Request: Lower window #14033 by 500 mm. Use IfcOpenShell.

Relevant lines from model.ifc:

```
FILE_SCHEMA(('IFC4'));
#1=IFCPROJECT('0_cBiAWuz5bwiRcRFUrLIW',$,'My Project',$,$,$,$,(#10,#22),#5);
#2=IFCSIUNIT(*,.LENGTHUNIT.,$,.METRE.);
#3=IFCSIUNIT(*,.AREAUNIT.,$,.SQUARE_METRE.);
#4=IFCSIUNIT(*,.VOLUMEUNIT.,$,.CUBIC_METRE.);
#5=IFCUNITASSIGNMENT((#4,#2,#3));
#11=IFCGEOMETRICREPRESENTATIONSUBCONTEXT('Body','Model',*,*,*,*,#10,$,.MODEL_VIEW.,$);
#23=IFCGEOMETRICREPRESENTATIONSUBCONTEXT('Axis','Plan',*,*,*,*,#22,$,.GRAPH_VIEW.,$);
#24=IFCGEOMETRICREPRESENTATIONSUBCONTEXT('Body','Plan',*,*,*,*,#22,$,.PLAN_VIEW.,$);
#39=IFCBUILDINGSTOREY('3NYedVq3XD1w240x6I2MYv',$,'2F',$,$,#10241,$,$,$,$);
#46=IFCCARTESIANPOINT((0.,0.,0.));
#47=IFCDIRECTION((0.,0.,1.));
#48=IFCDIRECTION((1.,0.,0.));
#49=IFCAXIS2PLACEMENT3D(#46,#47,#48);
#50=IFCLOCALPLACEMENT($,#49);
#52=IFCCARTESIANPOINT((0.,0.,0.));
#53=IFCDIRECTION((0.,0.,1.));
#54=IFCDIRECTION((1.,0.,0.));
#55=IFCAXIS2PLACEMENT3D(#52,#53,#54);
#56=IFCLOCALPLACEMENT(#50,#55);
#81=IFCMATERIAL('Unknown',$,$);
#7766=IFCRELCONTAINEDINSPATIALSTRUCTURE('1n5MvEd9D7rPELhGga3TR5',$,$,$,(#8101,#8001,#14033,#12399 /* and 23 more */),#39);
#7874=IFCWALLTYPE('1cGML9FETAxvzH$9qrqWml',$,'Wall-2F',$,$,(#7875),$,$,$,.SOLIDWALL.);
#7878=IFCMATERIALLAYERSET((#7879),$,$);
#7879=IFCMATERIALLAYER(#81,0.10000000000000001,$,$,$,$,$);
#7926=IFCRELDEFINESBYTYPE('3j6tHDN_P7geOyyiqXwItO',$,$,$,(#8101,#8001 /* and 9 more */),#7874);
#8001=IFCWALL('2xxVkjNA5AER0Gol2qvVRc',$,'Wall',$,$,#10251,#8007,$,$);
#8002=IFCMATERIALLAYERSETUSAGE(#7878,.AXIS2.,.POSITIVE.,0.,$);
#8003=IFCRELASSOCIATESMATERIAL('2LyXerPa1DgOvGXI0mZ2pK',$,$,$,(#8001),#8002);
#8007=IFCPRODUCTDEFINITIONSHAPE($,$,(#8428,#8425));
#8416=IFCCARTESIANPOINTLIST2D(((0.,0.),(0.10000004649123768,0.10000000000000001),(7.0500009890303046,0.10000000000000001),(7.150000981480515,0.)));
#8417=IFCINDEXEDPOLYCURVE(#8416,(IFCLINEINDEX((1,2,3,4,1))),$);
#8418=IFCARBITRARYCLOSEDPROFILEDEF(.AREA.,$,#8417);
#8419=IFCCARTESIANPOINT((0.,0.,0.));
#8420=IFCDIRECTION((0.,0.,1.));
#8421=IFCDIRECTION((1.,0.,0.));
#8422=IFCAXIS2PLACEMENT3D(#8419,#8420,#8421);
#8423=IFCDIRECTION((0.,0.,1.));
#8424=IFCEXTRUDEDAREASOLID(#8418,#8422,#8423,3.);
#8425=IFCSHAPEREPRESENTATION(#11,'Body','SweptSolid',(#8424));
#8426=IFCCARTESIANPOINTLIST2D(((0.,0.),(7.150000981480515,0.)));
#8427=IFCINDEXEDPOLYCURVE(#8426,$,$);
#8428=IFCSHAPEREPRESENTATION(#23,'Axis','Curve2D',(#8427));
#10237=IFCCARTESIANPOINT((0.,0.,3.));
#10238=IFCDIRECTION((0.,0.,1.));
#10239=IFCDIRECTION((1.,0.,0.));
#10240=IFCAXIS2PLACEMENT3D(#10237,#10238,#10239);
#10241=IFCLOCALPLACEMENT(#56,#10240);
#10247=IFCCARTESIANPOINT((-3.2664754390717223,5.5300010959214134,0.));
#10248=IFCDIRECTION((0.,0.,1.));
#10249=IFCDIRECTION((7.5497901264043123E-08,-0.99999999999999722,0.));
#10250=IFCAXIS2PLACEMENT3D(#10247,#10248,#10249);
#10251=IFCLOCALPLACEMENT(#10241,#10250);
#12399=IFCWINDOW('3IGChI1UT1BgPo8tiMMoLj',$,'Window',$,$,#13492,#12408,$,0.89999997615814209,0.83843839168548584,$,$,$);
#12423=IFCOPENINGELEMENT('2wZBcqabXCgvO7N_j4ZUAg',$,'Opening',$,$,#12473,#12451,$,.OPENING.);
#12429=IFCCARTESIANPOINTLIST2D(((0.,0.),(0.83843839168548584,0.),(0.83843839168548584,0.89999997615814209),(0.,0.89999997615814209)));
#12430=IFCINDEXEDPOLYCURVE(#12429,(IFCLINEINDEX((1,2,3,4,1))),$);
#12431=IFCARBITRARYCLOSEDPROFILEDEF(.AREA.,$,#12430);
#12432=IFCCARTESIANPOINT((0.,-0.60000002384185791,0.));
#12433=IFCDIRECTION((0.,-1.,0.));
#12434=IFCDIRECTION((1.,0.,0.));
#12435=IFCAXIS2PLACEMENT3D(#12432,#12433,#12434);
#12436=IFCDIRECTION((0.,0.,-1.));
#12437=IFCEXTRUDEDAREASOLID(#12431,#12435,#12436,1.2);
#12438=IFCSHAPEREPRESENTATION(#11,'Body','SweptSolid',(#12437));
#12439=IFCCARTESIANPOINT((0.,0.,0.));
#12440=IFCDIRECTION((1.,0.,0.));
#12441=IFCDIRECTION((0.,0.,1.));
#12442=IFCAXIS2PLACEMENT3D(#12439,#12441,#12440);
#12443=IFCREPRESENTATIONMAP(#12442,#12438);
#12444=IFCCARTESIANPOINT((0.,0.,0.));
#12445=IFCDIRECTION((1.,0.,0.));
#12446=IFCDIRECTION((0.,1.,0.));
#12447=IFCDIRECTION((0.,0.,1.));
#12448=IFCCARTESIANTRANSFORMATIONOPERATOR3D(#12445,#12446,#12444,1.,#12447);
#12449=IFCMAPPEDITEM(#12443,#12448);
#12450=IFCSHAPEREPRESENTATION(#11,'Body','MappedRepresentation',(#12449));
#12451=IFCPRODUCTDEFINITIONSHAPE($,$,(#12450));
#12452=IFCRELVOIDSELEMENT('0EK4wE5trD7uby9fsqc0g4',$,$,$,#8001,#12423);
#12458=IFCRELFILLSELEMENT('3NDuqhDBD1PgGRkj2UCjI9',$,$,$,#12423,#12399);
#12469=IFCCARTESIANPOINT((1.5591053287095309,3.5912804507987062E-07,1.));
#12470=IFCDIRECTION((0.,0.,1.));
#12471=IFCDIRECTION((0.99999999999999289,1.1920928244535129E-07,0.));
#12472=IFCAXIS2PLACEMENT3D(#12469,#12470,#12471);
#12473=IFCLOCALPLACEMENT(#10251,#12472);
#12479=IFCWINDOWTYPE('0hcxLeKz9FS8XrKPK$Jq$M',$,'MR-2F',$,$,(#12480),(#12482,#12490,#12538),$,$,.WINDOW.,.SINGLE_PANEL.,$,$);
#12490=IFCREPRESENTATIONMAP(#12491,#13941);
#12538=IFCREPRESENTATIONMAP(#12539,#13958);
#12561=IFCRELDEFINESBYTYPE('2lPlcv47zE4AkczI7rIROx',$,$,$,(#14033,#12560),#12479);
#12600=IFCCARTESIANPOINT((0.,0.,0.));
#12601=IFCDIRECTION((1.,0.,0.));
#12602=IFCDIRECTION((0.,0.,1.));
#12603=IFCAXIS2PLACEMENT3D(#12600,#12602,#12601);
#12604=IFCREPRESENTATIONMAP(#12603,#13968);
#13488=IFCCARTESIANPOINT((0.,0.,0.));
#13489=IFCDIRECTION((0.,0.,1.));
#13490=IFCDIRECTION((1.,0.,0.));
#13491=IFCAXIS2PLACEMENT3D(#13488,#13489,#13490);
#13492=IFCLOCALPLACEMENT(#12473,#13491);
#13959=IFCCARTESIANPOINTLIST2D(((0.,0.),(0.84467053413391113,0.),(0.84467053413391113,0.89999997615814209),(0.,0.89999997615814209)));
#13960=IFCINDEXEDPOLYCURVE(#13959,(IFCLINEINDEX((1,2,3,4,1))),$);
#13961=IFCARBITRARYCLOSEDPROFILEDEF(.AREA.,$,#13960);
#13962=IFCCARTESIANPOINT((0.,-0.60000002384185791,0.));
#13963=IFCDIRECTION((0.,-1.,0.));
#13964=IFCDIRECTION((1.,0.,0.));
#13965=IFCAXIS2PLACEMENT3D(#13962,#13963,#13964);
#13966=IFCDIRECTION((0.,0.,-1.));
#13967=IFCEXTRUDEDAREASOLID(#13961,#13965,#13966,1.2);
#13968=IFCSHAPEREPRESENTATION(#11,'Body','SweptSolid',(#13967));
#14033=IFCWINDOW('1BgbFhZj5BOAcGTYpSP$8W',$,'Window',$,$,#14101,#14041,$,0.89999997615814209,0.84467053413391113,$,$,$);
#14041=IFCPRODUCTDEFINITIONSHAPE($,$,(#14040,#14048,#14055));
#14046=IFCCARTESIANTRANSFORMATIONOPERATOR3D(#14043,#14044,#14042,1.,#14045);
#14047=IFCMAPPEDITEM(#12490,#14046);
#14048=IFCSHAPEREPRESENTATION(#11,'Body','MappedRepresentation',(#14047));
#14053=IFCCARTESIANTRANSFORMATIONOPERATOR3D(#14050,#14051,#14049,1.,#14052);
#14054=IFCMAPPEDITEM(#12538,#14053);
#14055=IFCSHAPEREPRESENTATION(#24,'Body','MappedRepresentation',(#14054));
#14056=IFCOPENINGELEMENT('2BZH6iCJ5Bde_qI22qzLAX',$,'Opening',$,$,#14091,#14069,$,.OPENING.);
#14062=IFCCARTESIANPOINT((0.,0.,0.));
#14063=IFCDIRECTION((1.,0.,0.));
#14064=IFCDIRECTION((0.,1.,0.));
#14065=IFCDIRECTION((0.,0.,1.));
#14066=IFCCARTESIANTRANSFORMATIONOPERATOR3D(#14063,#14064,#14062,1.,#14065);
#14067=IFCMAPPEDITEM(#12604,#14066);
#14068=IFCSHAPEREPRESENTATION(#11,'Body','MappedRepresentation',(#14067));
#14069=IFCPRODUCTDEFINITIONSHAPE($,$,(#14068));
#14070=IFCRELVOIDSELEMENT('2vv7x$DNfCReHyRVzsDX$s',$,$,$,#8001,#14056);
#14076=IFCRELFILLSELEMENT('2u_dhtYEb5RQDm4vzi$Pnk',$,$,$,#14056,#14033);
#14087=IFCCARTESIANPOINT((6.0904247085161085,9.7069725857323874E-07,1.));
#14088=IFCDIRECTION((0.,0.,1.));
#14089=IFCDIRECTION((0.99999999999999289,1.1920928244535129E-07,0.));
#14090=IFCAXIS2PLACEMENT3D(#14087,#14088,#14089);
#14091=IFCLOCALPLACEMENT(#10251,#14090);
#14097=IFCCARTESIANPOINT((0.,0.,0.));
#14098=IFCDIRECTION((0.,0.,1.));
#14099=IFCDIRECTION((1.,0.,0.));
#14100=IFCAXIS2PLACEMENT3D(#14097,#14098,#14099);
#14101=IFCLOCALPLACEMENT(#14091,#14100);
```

```python
import numpy as np
import ifcopenshell
import ifcopenshell.api.geometry
import ifcopenshell.util.placement
import ifcopenshell.util.unit

model = ifcopenshell.open("model.ifc")
unit_scale = ifcopenshell.util.unit.calculate_unit_scale(model)

window = model.by_id(14033)
opening = window.FillsVoids[0].RelatingOpeningElement
dz = -0.5

shift = np.array([0.0, 0.0, dz])
# The window is placed relative to its opening, so it follows when the opening moves.
matrix = ifcopenshell.util.placement.get_local_placement(opening.ObjectPlacement)
matrix[:3, 3] += shift
ifcopenshell.api.geometry.edit_object_placement(
    model, product=opening, matrix=matrix, is_si=False, should_transform_children=True
)

print(f"moved by {dz * unit_scale:+.3f} m")

model.write("model-out.ifc")
```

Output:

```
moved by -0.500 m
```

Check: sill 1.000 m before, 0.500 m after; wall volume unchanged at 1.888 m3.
